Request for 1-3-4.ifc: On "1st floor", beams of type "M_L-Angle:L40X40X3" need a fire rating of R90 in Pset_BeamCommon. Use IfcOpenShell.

First a look at what the model holds.

```python
import ifcopenshell
import ifcopenshell.util.element

model = ifcopenshell.open("1-3-4.ifc")
print(model.schema)
storey = next(s for s in model.by_type("IfcBuildingStorey") if s.Name == "1st floor")
beams = [e for e in ifcopenshell.util.element.get_decomposition(storey) if e.is_a("IfcBeam")]
seen = {}
for e in beams:
    element_type = ifcopenshell.util.element.get_type(e)
    key = (element_type.Name if element_type != e and element_type else None, ifcopenshell.util.element.get_pset(e, "Pset_BeamCommon", "FireRating"))
    seen[key] = seen.get(key, 0) + 1
for (name, value), count in sorted(seen.items(), key=str):
    print(count, "x", name, "|", value)
```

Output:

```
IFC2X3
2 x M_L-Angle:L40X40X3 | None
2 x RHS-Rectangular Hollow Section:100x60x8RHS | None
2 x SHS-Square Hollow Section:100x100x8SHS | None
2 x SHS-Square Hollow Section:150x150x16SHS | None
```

```python
import ifcopenshell
import ifcopenshell.api.pset
import ifcopenshell.util.element

model = ifcopenshell.open("1-3-4.ifc")

storey = next(s for s in model.by_type("IfcBuildingStorey") if s.Name == "1st floor")
beams = [e for e in ifcopenshell.util.element.get_decomposition(storey) if e.is_a("IfcBeam")]

count = 0
for e in beams:
    element_type = ifcopenshell.util.element.get_type(e)
    if element_type in (None, e) or element_type.Name != "M_L-Angle:L40X40X3":
        continue
    # add_pset returns the element's existing set when there is one.
    pset = ifcopenshell.api.pset.add_pset(model, product=e, name="Pset_BeamCommon")
    ifcopenshell.api.pset.edit_pset(model, pset=pset, properties={"FireRating": "R90"})
    count += 1

print(count, "beams updated")

model.write("1-3-4_updated.ifc")
```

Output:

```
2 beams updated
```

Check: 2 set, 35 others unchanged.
